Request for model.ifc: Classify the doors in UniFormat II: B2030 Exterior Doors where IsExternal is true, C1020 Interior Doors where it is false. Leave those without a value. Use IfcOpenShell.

First a look at what the model holds.

```python
import ifcopenshell
import ifcopenshell.util.element

model = ifcopenshell.open("model.ifc")
print(model.schema)
print("classifications:", [c.Name for c in model.by_type("IfcClassification")])
values = [ifcopenshell.util.element.get_pset(e, "Pset_DoorCommon", "IsExternal") for e in model.by_type("IfcDoor")]
for value in (True, False, None):
    print("IsExternal", value, values.count(value))
```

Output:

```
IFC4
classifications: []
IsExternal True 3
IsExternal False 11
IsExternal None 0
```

```python
import ifcopenshell
import ifcopenshell.api.classification
import ifcopenshell.util.element

model = ifcopenshell.open("model.ifc")

system = ifcopenshell.api.classification.add_classification(model, classification="UniFormat II")

doors = model.by_type("IfcDoor")
external = {e: ifcopenshell.util.element.get_pset(e, "Pset_DoorCommon", "IsExternal") for e in doors}
for flag, code, name in ((True, "B2030", "Exterior Doors"), (False, "C1020", "Interior Doors")):
    products = [e for e in doors if external[e] is flag]
    ifcopenshell.api.classification.add_reference(
        model, products=products, classification=system, identification=code, name=name
    )
    print(code, len(products))

model.write("model_updated.ifc")
```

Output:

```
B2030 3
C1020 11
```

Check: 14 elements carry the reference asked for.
